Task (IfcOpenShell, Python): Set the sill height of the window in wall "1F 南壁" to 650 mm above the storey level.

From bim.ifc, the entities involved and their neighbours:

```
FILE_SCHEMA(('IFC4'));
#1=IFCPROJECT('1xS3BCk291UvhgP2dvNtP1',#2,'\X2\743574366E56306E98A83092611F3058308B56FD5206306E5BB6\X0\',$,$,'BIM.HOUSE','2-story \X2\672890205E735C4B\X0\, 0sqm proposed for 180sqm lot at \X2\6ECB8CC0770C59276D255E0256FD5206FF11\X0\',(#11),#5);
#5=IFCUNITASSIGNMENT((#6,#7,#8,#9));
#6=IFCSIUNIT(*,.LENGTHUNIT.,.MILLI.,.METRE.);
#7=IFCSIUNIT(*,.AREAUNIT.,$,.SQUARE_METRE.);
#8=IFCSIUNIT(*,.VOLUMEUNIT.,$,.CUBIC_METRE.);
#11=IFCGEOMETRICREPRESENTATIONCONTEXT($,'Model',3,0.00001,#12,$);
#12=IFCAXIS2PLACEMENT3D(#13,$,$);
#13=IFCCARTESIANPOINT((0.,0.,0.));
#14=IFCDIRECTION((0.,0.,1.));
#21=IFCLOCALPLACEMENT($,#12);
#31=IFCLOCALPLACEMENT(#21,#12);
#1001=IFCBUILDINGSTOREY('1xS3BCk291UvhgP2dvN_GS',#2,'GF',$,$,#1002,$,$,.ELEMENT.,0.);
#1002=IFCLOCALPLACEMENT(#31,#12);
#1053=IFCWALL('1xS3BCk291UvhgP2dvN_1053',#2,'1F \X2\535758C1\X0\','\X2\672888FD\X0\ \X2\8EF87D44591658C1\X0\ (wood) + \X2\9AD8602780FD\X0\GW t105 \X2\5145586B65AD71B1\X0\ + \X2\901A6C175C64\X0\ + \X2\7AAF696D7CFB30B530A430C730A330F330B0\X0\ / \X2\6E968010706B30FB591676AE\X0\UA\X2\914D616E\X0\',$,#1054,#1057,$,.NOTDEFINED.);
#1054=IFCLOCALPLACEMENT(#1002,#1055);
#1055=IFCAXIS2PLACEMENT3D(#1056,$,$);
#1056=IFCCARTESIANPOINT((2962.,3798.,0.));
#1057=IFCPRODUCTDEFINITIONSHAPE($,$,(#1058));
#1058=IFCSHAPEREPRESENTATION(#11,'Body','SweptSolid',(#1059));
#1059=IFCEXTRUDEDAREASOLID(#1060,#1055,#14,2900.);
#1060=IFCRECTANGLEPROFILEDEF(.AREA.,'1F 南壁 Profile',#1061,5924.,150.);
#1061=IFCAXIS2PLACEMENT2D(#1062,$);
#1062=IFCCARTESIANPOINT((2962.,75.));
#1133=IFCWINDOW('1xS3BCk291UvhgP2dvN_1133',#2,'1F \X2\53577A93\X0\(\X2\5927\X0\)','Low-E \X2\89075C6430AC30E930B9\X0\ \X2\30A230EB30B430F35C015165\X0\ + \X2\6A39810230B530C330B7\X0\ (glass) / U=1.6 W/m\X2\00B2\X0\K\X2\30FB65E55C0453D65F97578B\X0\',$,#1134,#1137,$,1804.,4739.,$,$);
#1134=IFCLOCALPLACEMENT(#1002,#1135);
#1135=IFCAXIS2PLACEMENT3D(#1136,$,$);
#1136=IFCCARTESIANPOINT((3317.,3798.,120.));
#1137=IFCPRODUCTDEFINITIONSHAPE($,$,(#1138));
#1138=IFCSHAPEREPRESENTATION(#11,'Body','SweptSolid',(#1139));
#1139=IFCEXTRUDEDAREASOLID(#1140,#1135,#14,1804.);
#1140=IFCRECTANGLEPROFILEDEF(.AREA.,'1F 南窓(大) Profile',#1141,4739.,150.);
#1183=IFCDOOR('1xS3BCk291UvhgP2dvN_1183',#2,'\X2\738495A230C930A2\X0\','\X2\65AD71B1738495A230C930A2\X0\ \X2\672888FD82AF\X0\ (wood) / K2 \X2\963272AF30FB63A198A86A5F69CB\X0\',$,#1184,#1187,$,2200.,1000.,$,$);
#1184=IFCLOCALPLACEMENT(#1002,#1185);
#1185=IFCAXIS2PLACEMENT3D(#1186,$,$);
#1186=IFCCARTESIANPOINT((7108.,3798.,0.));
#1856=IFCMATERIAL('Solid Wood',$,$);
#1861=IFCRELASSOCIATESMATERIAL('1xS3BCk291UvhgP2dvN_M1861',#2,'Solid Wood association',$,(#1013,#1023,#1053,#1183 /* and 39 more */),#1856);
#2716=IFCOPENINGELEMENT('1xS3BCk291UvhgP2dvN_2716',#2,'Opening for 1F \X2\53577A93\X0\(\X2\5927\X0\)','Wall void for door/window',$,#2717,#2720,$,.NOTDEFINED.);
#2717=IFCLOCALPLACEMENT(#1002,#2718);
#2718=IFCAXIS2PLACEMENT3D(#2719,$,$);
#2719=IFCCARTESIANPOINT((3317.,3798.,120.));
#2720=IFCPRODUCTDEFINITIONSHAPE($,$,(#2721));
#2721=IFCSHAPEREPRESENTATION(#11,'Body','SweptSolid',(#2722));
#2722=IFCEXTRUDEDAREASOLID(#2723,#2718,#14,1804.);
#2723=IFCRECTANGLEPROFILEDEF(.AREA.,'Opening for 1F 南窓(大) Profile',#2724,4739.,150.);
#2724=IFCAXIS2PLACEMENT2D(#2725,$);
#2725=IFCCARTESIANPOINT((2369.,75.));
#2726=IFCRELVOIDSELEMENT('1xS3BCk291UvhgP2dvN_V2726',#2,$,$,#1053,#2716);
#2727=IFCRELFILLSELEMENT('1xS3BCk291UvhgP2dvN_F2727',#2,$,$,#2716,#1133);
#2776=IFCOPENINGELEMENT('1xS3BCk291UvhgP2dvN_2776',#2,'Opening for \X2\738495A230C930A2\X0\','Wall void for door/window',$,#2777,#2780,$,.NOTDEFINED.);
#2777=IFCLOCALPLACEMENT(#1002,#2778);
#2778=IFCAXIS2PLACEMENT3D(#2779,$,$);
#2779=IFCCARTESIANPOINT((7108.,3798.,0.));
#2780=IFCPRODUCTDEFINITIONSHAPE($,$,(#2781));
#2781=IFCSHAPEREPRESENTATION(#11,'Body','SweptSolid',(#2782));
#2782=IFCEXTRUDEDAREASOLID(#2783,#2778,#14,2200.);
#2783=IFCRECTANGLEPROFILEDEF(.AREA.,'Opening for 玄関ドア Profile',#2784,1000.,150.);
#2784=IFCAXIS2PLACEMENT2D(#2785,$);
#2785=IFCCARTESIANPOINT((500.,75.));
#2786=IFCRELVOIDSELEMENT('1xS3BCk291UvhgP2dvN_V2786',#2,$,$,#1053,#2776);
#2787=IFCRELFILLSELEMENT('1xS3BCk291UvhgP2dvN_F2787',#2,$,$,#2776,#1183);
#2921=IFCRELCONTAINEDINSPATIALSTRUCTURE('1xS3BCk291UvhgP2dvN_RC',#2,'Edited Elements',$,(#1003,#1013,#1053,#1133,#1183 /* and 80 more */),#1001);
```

```python
import numpy as np
import ifcopenshell
import ifcopenshell.api.geometry
import ifcopenshell.geom
import ifcopenshell.util.element
import ifcopenshell.util.placement
import ifcopenshell.util.shape
import ifcopenshell.util.unit

model = ifcopenshell.open("bim.ifc")
unit_scale = ifcopenshell.util.unit.calculate_unit_scale(model)

window = model.by_guid("1xS3BCk291UvhgP2dvN_1133")
opening = window.FillsVoids[0].RelatingOpeningElement
storey = ifcopenshell.util.element.get_container(window, ifc_class="IfcBuildingStorey")
level = ifcopenshell.util.placement.get_local_placement(storey.ObjectPlacement)[2, 3]

# The opening's origin need not be at the sill, so measure its lowest point.
shape = ifcopenshell.geom.create_shape(ifcopenshell.geom.settings(), opening)
bottom = ifcopenshell.util.shape.get_shape_bottom_elevation(shape, shape.geometry) / unit_scale
dz = level + 0.65 / unit_scale - bottom

shift = np.array([0.0, 0.0, dz])
# The window is not placed relative to its opening, so move both.
for product in (opening, window):
    matrix = ifcopenshell.util.placement.get_local_placement(product.ObjectPlacement)
    matrix[:3, 3] += shift
    ifcopenshell.api.geometry.edit_object_placement(model, product=product, matrix=matrix, is_si=False)

print(f"moved by {dz * unit_scale:+.3f} m")

model.write("bim_v2.ifc")
```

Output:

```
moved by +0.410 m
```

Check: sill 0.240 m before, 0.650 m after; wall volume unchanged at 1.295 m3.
